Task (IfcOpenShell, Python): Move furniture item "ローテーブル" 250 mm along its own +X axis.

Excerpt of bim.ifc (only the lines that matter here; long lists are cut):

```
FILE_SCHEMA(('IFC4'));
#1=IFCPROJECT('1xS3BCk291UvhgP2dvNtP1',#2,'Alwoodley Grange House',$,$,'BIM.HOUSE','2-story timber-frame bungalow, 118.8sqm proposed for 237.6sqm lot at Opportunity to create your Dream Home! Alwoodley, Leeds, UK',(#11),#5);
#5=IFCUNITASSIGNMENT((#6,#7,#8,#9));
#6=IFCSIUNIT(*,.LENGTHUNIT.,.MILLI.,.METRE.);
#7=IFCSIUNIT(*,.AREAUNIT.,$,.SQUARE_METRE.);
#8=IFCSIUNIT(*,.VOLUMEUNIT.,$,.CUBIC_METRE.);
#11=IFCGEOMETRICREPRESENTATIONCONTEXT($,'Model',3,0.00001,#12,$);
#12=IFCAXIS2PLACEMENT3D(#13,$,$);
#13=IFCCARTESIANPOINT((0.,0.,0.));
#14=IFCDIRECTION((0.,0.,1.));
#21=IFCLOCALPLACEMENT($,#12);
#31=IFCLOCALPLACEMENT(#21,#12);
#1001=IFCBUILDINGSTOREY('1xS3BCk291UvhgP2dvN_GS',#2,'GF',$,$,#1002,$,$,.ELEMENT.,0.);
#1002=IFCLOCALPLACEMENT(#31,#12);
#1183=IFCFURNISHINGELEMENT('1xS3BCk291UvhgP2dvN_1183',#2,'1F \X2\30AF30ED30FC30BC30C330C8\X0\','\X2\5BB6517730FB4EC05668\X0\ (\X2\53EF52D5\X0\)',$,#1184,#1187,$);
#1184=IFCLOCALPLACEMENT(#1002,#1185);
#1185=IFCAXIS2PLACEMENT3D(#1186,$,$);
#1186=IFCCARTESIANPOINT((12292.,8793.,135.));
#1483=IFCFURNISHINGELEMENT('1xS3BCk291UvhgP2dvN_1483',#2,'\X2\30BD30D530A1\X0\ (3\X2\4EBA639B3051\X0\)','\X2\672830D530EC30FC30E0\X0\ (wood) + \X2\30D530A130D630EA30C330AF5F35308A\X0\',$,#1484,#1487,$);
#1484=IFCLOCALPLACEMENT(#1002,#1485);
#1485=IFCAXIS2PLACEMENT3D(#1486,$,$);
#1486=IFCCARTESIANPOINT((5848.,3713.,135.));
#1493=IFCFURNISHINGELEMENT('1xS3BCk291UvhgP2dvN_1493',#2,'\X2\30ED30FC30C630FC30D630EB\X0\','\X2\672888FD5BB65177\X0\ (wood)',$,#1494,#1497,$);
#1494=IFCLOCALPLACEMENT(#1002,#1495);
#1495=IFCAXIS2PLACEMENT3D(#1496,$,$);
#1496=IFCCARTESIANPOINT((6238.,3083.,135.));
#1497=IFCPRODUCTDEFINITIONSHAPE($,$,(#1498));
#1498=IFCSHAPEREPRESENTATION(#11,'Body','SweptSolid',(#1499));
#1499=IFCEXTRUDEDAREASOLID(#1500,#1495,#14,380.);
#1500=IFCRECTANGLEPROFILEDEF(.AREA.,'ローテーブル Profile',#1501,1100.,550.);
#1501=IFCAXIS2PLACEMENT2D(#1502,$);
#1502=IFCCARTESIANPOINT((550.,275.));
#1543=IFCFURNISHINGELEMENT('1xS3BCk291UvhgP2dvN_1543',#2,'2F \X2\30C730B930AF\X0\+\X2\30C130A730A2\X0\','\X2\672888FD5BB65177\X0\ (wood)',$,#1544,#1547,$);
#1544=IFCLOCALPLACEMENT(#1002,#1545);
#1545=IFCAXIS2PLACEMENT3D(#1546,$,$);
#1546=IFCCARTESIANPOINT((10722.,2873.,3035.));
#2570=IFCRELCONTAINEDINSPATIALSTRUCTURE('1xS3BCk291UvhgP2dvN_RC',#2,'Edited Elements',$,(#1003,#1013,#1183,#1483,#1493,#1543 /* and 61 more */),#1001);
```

```python
import ifcopenshell
import ifcopenshell.api.geometry
import ifcopenshell.util.placement

model = ifcopenshell.open("bim.ifc")

item = model.by_guid("1xS3BCk291UvhgP2dvN_1493")
matrix = ifcopenshell.util.placement.get_local_placement(item.ObjectPlacement)
matrix[:3, 3] += matrix[:3, 0] * 250.0
ifcopenshell.api.geometry.edit_object_placement(model, product=item, matrix=matrix, is_si=False)

print(ifcopenshell.util.placement.get_local_placement(item.ObjectPlacement).round(3) + 0.0)

model.write("bim-out.ifc")
```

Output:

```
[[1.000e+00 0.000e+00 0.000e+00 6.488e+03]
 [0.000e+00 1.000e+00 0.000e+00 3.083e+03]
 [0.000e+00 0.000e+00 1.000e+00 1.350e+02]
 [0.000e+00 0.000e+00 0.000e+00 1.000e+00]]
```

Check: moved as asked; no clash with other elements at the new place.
